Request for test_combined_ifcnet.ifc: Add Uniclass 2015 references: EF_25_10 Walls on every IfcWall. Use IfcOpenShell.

First a look at what the model holds.

```python
import ifcopenshell

model = ifcopenshell.open("test_combined_ifcnet.ifc")
print(model.schema)
print("classifications:", [c.Name for c in model.by_type("IfcClassification")])
for ifc_class in ("IfcDoor", "IfcRoof", "IfcStair", "IfcWall", "IfcWindow"):
    print(ifc_class, len(model.by_type(ifc_class)))
```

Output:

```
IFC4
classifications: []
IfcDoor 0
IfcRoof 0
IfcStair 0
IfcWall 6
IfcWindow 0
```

```python
import ifcopenshell
import ifcopenshell.api.classification

model = ifcopenshell.open("test_combined_ifcnet.ifc")

system = ifcopenshell.api.classification.add_classification(model, classification="Uniclass 2015")

codes = {
    "IfcWall": ("EF_25_10", "Walls"),
}
for ifc_class, (code, name) in codes.items():
    products = model.by_type(ifc_class)
    ifcopenshell.api.classification.add_reference(
        model, products=products, classification=system, identification=code, name=name
    )
    print(code, len(products))

model.write("test_combined_ifcnet-out.ifc")
```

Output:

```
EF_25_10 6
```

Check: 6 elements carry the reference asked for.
